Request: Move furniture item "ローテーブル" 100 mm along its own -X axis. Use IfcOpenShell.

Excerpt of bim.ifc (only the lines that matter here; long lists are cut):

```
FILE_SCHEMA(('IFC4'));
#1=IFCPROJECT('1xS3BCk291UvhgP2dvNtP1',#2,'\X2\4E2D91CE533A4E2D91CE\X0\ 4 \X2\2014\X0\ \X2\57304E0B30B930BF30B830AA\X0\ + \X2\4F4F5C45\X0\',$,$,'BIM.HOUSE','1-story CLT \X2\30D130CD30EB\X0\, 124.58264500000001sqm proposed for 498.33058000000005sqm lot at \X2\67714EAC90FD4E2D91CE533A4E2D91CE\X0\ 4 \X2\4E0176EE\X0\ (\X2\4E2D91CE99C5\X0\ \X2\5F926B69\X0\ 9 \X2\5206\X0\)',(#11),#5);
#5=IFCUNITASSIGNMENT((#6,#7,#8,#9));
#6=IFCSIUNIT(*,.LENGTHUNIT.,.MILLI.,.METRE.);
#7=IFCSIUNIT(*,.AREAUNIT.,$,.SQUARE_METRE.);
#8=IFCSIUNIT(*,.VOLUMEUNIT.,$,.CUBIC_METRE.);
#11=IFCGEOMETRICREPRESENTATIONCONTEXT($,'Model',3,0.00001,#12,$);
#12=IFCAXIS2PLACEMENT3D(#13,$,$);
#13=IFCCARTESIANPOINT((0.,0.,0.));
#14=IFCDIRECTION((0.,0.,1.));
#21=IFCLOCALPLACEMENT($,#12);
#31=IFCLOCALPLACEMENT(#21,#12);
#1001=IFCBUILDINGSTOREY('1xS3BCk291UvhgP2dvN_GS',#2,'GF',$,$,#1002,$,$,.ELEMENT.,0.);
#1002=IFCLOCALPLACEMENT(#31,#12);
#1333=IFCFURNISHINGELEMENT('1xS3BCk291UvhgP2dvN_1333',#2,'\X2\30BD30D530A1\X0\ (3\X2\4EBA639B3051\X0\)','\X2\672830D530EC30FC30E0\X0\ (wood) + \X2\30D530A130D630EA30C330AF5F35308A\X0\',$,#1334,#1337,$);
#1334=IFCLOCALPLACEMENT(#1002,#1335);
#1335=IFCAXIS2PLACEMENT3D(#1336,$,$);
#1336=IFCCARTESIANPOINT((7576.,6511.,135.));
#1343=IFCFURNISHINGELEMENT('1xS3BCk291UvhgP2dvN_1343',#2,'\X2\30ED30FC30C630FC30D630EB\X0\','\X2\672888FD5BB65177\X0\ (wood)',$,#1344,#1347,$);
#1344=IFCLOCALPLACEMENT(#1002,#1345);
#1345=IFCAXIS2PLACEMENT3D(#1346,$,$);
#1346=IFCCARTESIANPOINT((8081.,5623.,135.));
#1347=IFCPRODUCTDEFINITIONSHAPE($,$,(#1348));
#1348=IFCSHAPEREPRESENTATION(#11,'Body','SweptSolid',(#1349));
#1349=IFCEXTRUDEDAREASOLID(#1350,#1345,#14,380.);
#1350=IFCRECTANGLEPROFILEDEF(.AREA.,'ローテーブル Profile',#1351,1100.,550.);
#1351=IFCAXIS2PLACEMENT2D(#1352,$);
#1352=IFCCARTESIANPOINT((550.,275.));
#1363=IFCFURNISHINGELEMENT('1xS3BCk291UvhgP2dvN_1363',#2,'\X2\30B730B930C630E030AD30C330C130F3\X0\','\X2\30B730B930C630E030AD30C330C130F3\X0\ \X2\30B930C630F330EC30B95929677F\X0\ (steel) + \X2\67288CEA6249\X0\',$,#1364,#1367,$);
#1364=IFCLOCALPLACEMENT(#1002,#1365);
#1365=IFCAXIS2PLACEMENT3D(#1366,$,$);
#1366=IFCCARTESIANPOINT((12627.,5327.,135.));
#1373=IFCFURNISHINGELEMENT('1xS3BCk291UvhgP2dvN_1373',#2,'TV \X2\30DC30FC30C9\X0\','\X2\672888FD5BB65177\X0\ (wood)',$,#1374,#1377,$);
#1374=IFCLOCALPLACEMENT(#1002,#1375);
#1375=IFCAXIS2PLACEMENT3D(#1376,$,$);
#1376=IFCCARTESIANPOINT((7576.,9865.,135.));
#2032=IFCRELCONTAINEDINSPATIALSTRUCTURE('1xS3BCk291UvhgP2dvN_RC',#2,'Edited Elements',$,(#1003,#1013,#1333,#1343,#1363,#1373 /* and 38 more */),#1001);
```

```python
import ifcopenshell
import ifcopenshell.api.geometry
import ifcopenshell.util.placement
import ifcopenshell.util.unit

model = ifcopenshell.open("bim.ifc")
unit_scale = ifcopenshell.util.unit.calculate_unit_scale(model)

item = model.by_guid("1xS3BCk291UvhgP2dvN_1343")
matrix = ifcopenshell.util.placement.get_local_placement(item.ObjectPlacement)
matrix[:3, 3] -= matrix[:3, 0] * 0.1 / unit_scale
ifcopenshell.api.geometry.edit_object_placement(model, product=item, matrix=matrix, is_si=False)

print(ifcopenshell.util.placement.get_local_placement(item.ObjectPlacement).round(3) + 0.0)

model.write("bim_updated.ifc")
```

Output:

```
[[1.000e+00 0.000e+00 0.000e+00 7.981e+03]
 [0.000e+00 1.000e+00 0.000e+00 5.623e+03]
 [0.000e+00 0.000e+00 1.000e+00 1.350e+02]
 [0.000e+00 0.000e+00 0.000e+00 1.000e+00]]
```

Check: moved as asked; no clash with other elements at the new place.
